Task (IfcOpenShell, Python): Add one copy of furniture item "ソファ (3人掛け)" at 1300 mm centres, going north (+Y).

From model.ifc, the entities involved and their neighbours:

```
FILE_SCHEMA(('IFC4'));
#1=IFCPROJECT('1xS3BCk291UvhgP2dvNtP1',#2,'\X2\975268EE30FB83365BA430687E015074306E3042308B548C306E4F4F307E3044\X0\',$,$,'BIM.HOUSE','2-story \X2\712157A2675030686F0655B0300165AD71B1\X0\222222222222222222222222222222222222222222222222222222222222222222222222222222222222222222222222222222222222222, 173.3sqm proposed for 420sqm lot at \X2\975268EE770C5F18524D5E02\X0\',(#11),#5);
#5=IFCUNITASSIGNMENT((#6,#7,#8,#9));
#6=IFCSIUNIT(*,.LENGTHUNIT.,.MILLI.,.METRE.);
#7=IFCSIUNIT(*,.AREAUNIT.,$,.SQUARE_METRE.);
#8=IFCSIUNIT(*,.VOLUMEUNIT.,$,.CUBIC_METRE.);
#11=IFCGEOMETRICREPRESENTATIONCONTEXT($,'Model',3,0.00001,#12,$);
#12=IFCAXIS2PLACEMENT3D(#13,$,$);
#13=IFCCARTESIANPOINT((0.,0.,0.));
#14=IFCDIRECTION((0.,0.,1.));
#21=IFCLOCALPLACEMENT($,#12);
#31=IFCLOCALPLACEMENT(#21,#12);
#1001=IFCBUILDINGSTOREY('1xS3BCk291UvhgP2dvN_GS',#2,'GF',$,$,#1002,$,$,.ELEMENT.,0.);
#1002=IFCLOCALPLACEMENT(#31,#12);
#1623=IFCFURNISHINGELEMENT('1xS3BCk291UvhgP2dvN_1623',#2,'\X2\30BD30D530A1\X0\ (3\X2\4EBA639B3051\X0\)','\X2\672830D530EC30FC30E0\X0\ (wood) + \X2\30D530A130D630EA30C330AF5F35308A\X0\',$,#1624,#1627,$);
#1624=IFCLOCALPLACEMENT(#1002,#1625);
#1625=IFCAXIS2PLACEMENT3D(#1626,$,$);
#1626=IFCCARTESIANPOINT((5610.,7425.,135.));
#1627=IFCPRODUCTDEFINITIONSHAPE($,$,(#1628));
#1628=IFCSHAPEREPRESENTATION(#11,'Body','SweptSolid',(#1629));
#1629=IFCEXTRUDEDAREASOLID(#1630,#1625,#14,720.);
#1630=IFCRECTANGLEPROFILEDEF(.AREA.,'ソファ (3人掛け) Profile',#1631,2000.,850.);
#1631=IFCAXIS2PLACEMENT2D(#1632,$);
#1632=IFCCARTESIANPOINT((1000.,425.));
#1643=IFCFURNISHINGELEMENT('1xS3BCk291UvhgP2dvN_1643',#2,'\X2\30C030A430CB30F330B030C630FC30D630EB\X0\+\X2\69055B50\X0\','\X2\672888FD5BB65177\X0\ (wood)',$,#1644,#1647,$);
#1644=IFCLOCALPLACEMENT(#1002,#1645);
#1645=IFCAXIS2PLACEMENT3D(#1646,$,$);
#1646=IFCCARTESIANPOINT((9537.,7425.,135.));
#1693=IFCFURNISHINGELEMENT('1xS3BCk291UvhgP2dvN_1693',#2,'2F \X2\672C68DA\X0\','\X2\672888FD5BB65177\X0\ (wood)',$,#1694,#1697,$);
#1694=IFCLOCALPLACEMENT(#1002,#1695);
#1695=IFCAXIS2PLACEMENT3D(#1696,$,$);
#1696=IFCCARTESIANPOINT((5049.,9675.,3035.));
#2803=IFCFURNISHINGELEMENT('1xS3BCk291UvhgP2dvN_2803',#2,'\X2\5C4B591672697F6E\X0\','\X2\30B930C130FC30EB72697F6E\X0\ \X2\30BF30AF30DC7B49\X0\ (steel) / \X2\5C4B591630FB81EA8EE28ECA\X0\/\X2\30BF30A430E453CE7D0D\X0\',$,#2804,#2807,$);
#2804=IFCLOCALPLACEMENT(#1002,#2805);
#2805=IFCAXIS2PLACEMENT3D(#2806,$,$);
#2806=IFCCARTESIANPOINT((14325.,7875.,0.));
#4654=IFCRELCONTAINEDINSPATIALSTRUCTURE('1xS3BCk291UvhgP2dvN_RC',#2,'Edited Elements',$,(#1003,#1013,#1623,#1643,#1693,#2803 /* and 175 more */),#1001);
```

```python
import numpy as np
import ifcopenshell
import ifcopenshell.api.geometry
import ifcopenshell.api.root
import ifcopenshell.util.element
import ifcopenshell.util.placement

model = ifcopenshell.open("model.ifc")


def reuse_history(source, copy):
    """copy_class also copies each property set's owner history, people and application; keep the originals."""
    for rel in copy.IsDefinedBy:
        if rel.is_a("IfcRelDefinesByProperties") and (history := rel.RelatingPropertyDefinition.OwnerHistory):
            rel.RelatingPropertyDefinition.OwnerHistory = source.OwnerHistory
            ifcopenshell.util.element.remove_deep2(model, history)


source = model.by_id(1623)
base = ifcopenshell.util.placement.get_local_placement(source.ObjectPlacement)
step = np.array([0.0, 1.0, 0.0]) * 1300.0

for i in range(1, 2):
    copy = ifcopenshell.api.root.copy_class(model, product=source)
    copy.Representation = ifcopenshell.util.element.copy_deep(
        model, source.Representation, exclude=["IfcGeometricRepresentationContext", "IfcRepresentationMap"]
    )
    reuse_history(source, copy)
    matrix = base.copy()
    matrix[:3, 3] += i * step
    print("added at", matrix[:3, 3].round(3) + 0.0)
    ifcopenshell.api.geometry.edit_object_placement(model, product=copy, matrix=matrix, is_si=False)

model.write("model_v2.ifc")
```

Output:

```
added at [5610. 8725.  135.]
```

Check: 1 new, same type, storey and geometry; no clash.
